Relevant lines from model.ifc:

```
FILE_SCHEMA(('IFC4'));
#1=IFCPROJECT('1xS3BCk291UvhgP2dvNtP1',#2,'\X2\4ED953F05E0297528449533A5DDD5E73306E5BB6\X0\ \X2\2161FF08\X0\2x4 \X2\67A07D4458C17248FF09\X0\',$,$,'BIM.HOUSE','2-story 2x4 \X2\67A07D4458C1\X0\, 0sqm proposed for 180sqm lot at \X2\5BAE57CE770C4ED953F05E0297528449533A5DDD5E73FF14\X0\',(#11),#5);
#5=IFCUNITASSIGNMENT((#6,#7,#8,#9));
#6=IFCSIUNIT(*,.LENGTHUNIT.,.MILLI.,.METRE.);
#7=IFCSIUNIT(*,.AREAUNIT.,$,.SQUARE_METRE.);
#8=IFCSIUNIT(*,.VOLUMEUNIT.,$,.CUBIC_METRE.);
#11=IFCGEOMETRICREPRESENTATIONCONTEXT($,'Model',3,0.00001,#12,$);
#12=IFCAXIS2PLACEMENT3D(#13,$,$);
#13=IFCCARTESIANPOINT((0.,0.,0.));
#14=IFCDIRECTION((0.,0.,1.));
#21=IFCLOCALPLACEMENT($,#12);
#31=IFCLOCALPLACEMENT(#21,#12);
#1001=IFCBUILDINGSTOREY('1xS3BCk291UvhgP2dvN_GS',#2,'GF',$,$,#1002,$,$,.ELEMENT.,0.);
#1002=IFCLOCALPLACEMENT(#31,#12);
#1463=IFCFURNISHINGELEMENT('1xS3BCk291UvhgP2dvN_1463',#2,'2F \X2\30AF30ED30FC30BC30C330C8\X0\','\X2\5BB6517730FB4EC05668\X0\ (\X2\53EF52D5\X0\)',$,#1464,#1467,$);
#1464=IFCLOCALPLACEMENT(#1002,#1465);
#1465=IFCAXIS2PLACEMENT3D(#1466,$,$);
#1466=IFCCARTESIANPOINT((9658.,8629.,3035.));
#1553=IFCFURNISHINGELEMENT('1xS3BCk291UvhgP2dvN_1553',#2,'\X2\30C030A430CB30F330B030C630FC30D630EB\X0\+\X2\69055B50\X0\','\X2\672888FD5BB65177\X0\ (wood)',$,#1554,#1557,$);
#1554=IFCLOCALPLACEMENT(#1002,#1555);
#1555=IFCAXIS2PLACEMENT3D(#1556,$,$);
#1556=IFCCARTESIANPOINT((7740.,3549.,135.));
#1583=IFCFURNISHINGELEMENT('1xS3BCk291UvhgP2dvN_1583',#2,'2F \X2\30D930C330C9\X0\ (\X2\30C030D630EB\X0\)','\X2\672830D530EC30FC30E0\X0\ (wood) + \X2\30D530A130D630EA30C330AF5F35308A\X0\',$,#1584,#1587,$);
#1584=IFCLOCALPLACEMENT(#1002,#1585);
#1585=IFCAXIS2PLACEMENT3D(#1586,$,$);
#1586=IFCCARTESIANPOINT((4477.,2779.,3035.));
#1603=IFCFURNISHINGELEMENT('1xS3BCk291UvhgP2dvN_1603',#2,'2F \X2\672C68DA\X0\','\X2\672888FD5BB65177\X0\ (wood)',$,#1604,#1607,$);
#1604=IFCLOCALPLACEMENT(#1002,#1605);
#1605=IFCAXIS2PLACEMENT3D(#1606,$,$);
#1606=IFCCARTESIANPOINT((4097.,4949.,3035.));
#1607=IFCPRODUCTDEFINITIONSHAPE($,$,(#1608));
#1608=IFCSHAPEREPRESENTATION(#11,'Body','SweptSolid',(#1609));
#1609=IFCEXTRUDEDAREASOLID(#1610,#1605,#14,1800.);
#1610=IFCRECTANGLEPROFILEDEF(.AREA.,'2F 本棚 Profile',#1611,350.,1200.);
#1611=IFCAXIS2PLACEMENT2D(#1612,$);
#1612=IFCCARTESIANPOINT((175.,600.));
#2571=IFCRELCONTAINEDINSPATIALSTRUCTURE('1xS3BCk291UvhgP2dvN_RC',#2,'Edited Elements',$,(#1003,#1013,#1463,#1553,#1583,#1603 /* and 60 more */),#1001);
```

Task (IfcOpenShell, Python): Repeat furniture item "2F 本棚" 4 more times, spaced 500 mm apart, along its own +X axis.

```python
import ifcopenshell
import ifcopenshell.api.geometry
import ifcopenshell.api.root
import ifcopenshell.util.element
import ifcopenshell.util.placement

model = ifcopenshell.open("model.ifc")


def reuse_history(source, copy):
    """copy_class also copies each property set's owner history, people and application; keep the originals."""
    for rel in copy.IsDefinedBy:
        if rel.is_a("IfcRelDefinesByProperties") and (history := rel.RelatingPropertyDefinition.OwnerHistory):
            rel.RelatingPropertyDefinition.OwnerHistory = source.OwnerHistory
            ifcopenshell.util.element.remove_deep2(model, history)


source = model.by_guid("1xS3BCk291UvhgP2dvN_1603")
base = ifcopenshell.util.placement.get_local_placement(source.ObjectPlacement)
step = base[:3, 0] * 500.0

for i in range(1, 5):
    copy = ifcopenshell.api.root.copy_class(model, product=source)
    copy.Representation = ifcopenshell.util.element.copy_deep(
        model, source.Representation, exclude=["IfcGeometricRepresentationContext", "IfcRepresentationMap"]
    )
    reuse_history(source, copy)
    matrix = base.copy()
    matrix[:3, 3] += i * step
    print("added at", matrix[:3, 3].round(3) + 0.0)
    ifcopenshell.api.geometry.edit_object_placement(model, product=copy, matrix=matrix, is_si=False)

model.write("model_v2.ifc")
```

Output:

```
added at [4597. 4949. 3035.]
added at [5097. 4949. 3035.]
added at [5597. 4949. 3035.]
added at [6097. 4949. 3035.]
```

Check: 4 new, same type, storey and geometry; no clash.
